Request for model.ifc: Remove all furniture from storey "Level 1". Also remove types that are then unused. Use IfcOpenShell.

First a look at what the model holds.

```python
import ifcopenshell
import ifcopenshell.util.element

model = ifcopenshell.open("model.ifc")
print(model.schema)
storey = next(s for s in model.by_type("IfcBuildingStorey") if s.Name == "Level 1")
furniture = [e for e in ifcopenshell.util.element.get_decomposition(storey) if e.is_a("IfcFurnishingElement")]
seen = {}
for e in furniture:
    element_type = ifcopenshell.util.element.get_type(e)
    name = element_type.Name if element_type not in (None, e) else None
    seen[name] = seen.get(name, 0) + 1
for name, count in sorted(seen.items(), key=str):
    print(count, "x", name)
```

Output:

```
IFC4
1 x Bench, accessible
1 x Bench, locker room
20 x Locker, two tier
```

```python
import ifcopenshell
import ifcopenshell.api.root
import ifcopenshell.util.element

model = ifcopenshell.open("model.ifc")

storey = next(s for s in model.by_type("IfcBuildingStorey") if s.Name == "Level 1")
furniture = [e for e in ifcopenshell.util.element.get_decomposition(storey) if e.is_a("IfcFurnishingElement")]
types = {ifcopenshell.util.element.get_type(e) for e in furniture} - {None, *furniture}

for e in furniture:
    ifcopenshell.api.root.remove_product(model, product=e)
print(len(furniture), "removed")

unused = [t for t in types if not ifcopenshell.util.element.get_types(t)]
for t in unused:
    ifcopenshell.api.root.remove_product(model, product=t)
print(len(unused), "unused types removed")

model.write("model-out.ifc")
```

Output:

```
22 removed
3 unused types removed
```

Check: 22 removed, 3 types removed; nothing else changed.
